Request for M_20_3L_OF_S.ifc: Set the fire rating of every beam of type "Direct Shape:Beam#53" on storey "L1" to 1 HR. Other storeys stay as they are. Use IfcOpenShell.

First a look at what the model holds.

```python
import ifcopenshell
import ifcopenshell.util.element

model = ifcopenshell.open("M_20_3L_OF_S.ifc")
print(model.schema)
storey = next(s for s in model.by_type("IfcBuildingStorey") if s.Name == "L1")
beams = [e for e in ifcopenshell.util.element.get_decomposition(storey) if e.is_a("IfcBeam")]
seen = {}
for e in beams:
    element_type = ifcopenshell.util.element.get_type(e)
    key = (element_type.Name if element_type != e and element_type else None, ifcopenshell.util.element.get_pset(e, "Pset_BeamCommon", "FireRating"))
    seen[key] = seen.get(key, 0) + 1
for (name, value), count in sorted(seen.items(), key=str):
    print(count, "x", name, "|", value)
```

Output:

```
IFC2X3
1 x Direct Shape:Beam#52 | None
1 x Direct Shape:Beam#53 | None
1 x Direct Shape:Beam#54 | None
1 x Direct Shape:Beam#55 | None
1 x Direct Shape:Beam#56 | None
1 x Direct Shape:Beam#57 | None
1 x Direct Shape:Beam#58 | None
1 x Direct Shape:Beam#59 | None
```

```python
import ifcopenshell
import ifcopenshell.api.pset
import ifcopenshell.util.element

model = ifcopenshell.open("M_20_3L_OF_S.ifc")

storey = next(s for s in model.by_type("IfcBuildingStorey") if s.Name == "L1")
beams = [e for e in ifcopenshell.util.element.get_decomposition(storey) if e.is_a("IfcBeam")]

count = 0
for e in beams:
    element_type = ifcopenshell.util.element.get_type(e)
    if element_type in (None, e) or element_type.Name != "Direct Shape:Beam#53":
        continue
    # add_pset returns the element's existing set when there is one.
    pset = ifcopenshell.api.pset.add_pset(model, product=e, name="Pset_BeamCommon")
    ifcopenshell.api.pset.edit_pset(model, pset=pset, properties={"FireRating": "1 HR"})
    count += 1

print(count, "beams updated")

model.write("M_20_3L_OF_S_edited.ifc")
```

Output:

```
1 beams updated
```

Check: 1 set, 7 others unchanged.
